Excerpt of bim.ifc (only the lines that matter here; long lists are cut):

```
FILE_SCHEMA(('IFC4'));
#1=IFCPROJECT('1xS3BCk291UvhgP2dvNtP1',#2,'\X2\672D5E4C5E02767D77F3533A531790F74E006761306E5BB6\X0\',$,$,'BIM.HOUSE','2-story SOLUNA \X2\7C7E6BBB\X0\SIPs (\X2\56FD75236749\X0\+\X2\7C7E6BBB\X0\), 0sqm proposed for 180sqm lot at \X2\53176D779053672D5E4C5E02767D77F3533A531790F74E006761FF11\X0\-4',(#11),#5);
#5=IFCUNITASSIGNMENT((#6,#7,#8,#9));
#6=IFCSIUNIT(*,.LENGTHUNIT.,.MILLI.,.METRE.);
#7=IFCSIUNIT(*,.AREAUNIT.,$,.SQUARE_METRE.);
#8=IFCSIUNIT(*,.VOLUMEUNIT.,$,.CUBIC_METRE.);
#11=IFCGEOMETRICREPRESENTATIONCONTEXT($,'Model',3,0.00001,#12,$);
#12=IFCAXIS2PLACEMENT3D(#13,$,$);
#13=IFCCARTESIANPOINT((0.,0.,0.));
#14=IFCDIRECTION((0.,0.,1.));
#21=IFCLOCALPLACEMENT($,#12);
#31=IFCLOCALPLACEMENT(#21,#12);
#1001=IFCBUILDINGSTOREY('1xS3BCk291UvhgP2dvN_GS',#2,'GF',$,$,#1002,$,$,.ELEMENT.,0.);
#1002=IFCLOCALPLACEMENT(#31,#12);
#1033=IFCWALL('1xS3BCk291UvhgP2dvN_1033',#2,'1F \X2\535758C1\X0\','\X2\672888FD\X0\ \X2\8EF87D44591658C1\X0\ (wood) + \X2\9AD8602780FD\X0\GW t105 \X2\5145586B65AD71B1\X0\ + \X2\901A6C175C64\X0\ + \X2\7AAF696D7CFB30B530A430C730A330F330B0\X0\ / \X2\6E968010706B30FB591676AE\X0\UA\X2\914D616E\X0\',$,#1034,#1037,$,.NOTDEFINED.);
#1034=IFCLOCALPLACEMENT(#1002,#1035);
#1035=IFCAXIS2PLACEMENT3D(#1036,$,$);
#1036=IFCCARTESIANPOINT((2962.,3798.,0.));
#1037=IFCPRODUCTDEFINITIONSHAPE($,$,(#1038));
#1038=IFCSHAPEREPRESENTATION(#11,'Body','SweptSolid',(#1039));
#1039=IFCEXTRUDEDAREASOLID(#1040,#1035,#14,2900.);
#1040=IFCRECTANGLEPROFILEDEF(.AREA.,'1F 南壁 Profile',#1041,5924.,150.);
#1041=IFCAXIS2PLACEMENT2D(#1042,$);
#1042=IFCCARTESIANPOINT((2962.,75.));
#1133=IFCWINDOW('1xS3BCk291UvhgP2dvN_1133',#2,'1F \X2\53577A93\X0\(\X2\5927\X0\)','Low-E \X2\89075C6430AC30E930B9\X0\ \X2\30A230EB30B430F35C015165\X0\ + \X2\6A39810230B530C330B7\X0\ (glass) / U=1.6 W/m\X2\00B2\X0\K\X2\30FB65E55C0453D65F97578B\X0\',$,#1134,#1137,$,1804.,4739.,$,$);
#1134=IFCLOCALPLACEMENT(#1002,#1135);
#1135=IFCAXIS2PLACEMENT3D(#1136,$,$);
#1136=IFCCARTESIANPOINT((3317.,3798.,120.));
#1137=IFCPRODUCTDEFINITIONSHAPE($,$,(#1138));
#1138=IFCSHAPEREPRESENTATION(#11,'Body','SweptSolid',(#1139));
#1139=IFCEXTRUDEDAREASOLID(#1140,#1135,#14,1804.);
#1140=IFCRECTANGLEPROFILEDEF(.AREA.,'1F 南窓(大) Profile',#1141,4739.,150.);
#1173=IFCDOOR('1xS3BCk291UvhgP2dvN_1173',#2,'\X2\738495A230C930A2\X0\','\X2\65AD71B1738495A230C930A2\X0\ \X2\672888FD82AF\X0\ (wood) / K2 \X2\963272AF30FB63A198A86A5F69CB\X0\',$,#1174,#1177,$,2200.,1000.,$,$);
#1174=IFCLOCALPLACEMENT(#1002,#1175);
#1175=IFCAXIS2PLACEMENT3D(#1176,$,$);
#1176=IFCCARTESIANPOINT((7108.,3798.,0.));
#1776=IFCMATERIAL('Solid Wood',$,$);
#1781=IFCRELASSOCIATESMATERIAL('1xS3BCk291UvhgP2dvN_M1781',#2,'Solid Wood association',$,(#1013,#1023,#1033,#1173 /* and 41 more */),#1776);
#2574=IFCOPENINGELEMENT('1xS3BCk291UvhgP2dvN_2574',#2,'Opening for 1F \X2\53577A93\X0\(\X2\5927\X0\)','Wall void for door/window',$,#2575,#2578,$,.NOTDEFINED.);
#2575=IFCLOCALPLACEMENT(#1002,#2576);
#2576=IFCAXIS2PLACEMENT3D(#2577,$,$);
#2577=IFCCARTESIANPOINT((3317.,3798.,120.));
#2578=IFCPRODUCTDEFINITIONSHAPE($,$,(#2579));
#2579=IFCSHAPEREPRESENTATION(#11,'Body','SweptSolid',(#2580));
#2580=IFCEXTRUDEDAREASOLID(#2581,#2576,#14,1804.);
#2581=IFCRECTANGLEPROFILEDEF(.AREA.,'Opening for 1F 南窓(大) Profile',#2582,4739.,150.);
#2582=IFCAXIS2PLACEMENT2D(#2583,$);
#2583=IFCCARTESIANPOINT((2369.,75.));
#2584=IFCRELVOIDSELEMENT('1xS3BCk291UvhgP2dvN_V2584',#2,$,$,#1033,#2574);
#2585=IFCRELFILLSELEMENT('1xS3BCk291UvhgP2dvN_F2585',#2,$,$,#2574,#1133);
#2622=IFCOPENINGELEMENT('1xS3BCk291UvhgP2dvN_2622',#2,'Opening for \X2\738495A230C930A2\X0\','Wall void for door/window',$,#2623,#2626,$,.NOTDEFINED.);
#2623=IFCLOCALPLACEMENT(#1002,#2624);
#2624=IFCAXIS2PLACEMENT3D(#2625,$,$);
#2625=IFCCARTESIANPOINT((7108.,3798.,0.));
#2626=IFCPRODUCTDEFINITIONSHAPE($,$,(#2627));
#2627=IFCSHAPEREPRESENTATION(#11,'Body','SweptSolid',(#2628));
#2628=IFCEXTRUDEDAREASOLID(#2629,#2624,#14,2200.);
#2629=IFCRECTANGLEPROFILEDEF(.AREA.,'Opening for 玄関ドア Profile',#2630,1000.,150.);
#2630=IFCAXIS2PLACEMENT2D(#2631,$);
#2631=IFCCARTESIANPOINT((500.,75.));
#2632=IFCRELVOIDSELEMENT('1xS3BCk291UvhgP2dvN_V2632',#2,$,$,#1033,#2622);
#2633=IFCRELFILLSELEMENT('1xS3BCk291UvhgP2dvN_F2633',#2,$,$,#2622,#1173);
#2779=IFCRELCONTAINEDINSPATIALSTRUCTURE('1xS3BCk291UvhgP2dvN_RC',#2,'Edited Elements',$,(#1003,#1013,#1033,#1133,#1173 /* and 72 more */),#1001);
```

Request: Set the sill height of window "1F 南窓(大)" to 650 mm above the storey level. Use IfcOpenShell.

```python
import numpy as np
import ifcopenshell
import ifcopenshell.api.geometry
import ifcopenshell.geom
import ifcopenshell.util.element
import ifcopenshell.util.placement
import ifcopenshell.util.shape
import ifcopenshell.util.unit

model = ifcopenshell.open("bim.ifc")
unit_scale = ifcopenshell.util.unit.calculate_unit_scale(model)

window = model.by_guid("1xS3BCk291UvhgP2dvN_1133")
opening = window.FillsVoids[0].RelatingOpeningElement
storey = ifcopenshell.util.element.get_container(window, ifc_class="IfcBuildingStorey")
level = ifcopenshell.util.placement.get_local_placement(storey.ObjectPlacement)[2, 3]

# The opening's origin need not be at the sill, so measure its lowest point.
shape = ifcopenshell.geom.create_shape(ifcopenshell.geom.settings(), opening)
bottom = ifcopenshell.util.shape.get_shape_bottom_elevation(shape, shape.geometry) / unit_scale
dz = level + 0.65 / unit_scale - bottom

shift = np.array([0.0, 0.0, dz])
# The window is not placed relative to its opening, so move both.
for product in (opening, window):
    matrix = ifcopenshell.util.placement.get_local_placement(product.ObjectPlacement)
    matrix[:3, 3] += shift
    ifcopenshell.api.geometry.edit_object_placement(model, product=product, matrix=matrix, is_si=False)

print(f"moved by {dz * unit_scale:+.3f} m")

model.write("bim_v2.ifc")
```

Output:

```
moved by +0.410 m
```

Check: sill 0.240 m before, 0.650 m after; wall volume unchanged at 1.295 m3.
